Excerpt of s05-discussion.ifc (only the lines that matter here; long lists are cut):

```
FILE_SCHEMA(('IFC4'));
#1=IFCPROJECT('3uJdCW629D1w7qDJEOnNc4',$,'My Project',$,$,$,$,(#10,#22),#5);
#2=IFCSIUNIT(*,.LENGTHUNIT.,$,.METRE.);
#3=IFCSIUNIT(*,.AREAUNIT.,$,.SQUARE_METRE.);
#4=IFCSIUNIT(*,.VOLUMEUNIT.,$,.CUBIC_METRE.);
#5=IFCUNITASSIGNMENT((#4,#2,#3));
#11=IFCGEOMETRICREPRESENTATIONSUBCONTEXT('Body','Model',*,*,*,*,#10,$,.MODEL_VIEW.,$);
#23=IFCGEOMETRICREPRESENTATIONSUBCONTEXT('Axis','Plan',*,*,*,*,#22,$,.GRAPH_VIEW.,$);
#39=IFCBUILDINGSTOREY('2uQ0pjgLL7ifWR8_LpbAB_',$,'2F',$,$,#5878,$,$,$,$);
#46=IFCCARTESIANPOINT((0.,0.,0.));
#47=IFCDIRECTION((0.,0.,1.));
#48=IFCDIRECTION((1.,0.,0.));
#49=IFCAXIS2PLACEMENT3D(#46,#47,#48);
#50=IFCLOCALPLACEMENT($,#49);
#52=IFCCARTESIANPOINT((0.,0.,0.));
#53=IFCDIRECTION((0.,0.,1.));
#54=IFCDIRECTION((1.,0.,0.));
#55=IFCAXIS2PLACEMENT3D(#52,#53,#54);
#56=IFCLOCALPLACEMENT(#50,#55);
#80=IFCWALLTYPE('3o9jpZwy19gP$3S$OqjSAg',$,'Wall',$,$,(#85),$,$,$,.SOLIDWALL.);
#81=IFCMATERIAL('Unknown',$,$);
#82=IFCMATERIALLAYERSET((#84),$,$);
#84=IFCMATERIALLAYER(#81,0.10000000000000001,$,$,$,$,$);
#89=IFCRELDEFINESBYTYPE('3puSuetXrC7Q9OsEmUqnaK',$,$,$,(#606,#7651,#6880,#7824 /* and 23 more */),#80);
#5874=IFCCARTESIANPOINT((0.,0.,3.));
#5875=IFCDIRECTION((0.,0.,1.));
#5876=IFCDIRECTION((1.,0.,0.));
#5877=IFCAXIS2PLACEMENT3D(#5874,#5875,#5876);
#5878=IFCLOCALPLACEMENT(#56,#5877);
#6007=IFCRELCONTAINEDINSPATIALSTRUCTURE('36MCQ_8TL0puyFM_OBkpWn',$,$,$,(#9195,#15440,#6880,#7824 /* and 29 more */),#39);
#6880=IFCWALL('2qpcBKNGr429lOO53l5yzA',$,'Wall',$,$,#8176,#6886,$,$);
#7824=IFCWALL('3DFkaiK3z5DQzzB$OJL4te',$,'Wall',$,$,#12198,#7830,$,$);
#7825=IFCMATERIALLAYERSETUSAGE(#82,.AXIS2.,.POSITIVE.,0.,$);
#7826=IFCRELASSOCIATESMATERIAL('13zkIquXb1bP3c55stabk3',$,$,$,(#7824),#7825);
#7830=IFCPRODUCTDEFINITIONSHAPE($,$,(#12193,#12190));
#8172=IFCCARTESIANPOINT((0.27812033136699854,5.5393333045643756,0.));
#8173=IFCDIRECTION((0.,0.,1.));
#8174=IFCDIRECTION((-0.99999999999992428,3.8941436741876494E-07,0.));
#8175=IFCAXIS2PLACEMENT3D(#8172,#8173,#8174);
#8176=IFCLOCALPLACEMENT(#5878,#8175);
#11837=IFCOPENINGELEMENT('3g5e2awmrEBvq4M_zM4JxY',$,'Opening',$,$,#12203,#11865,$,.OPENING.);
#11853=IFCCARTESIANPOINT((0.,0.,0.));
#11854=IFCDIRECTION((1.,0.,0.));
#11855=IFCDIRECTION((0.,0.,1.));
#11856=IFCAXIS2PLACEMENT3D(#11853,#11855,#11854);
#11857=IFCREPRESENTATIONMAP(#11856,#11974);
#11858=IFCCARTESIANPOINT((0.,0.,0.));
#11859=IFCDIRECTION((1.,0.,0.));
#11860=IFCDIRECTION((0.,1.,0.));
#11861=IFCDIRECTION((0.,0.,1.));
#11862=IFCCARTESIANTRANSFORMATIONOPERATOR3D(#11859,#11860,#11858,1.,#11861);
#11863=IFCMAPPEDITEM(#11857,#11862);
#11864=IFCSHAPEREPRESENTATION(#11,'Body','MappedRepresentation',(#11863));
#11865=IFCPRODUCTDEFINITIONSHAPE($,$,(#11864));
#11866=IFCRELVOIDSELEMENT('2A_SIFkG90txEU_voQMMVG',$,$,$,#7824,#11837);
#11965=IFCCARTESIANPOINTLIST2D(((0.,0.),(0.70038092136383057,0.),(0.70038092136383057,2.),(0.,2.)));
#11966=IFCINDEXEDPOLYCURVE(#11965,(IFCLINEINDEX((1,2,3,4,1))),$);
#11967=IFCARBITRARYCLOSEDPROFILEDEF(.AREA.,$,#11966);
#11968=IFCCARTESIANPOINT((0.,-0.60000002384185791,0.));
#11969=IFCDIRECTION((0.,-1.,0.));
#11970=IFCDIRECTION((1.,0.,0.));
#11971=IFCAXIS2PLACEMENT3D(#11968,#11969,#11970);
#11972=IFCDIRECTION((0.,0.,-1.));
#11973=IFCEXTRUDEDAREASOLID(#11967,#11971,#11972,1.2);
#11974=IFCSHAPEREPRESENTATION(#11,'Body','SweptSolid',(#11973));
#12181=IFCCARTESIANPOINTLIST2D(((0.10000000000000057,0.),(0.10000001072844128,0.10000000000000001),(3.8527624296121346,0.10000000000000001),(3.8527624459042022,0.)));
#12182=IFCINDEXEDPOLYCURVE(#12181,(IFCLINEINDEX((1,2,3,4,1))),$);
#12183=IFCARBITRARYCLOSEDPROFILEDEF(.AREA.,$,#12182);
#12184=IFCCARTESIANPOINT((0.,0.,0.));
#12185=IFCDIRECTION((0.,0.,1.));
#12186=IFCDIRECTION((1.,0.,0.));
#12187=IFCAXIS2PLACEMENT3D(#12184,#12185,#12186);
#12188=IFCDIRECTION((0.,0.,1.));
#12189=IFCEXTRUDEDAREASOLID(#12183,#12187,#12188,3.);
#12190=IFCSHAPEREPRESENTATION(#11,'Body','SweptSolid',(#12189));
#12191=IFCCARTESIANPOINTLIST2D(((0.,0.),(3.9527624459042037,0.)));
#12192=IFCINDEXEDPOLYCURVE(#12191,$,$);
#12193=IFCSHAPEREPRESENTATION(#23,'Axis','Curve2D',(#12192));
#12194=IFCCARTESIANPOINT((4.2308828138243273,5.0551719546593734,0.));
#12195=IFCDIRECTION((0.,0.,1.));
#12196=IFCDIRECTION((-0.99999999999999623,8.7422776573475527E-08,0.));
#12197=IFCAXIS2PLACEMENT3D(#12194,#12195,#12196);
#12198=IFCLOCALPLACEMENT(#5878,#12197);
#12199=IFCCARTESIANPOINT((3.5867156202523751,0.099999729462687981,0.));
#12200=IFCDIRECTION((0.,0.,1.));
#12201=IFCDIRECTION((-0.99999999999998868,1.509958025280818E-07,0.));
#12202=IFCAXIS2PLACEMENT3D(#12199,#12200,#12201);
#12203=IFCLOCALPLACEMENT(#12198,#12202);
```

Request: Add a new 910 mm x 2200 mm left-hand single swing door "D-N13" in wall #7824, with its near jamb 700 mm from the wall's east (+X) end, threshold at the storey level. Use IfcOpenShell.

```python
import numpy as np
import ifcopenshell
import ifcopenshell.api.feature
import ifcopenshell.api.geometry
import ifcopenshell.api.root
import ifcopenshell.api.spatial
import ifcopenshell.geom
import ifcopenshell.util.element
import ifcopenshell.util.placement
import ifcopenshell.util.representation
import ifcopenshell.util.shape
import ifcopenshell.util.unit

model = ifcopenshell.open("s05-discussion.ifc")
unit_scale = ifcopenshell.util.unit.calculate_unit_scale(model)
settings = ifcopenshell.geom.settings()


def volume(element):
    """Net volume in cubic metres, openings subtracted."""
    shape = ifcopenshell.geom.create_shape(settings, element)
    return ifcopenshell.util.shape.get_volume(shape.geometry)


wall = model.by_guid("3DFkaiK3z5DQzzB$OJL4te")
storey = ifcopenshell.util.element.get_container(wall, ifc_class="IfcBuildingStorey")
context = ifcopenshell.util.representation.get_context(model, "Model", "Body", "MODEL_VIEW")
before = volume(wall)

width, height, from_end, sill = 0.91, 2.2, 0.7, 0.0  # metres

# The wall runs along its own X axis, and the end named is its -X end.
wall_shape = ifcopenshell.geom.create_shape(settings, wall)
x, y, z = ifcopenshell.util.shape.get_vertices(wall_shape.geometry).T
start = x.min() + from_end
face, thickness = float(y.min()), float(y.max() - y.min())
wall_matrix = ifcopenshell.util.placement.get_local_placement(wall.ObjectPlacement)
level = ifcopenshell.util.placement.get_local_placement(storey.ObjectPlacement)[2, 3]


def in_wall(x, y):
    """Placement at x, y metres in the wall's axes, at sill height."""
    matrix = wall_matrix.copy()
    matrix[:, 3] = wall_matrix @ np.array([x / unit_scale, y / unit_scale, 0.0, 1.0])
    matrix[2, 3] = level + sill / unit_scale
    return matrix


# Opening: a box that overshoots both wall faces by 50 mm.
opening = ifcopenshell.api.root.create_entity(model, ifc_class="IfcOpeningElement", predefined_type="OPENING")
box = ifcopenshell.api.geometry.add_wall_representation(
    model, context=context, length=width, height=height, thickness=thickness + 0.1
)
ifcopenshell.api.geometry.assign_representation(model, product=opening, representation=box)
ifcopenshell.api.geometry.edit_object_placement(model, product=opening, matrix=in_wall(start, face - 0.05), is_si=False)
ifcopenshell.api.feature.add_feature(model, feature=opening, element=wall)

door = ifcopenshell.api.root.create_entity(model, ifc_class="IfcDoor", name="D-N13", predefined_type="DOOR")
door.OverallWidth, door.OverallHeight = width / unit_scale, height / unit_scale
door.OperationType = "SINGLE_SWING_LEFT"
body = ifcopenshell.api.geometry.add_door_representation(
    model,
    context=context,
    overall_width=door.OverallWidth,
    overall_height=door.OverallHeight,
    operation_type="SINGLE_SWING_LEFT",
    lining_properties={"LiningDepth": thickness / unit_scale, "ThresholdDepth": thickness / unit_scale},
)
ifcopenshell.api.geometry.assign_representation(model, product=door, representation=body)
ifcopenshell.api.spatial.assign_container(model, products=[door], relating_structure=storey)
ifcopenshell.api.feature.add_filling(model, opening=opening, element=door)

# The lining spans the wall, so the door starts at the wall face.
ifcopenshell.api.geometry.edit_object_placement(model, product=door, matrix=in_wall(start, face), is_si=False)

after = volume(wall)

print(f"wall volume {before:.3f} -> {after:.3f} m3")

model.write("s05-discussion-out.ifc")
```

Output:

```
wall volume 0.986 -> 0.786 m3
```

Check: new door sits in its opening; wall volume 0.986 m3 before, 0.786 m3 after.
